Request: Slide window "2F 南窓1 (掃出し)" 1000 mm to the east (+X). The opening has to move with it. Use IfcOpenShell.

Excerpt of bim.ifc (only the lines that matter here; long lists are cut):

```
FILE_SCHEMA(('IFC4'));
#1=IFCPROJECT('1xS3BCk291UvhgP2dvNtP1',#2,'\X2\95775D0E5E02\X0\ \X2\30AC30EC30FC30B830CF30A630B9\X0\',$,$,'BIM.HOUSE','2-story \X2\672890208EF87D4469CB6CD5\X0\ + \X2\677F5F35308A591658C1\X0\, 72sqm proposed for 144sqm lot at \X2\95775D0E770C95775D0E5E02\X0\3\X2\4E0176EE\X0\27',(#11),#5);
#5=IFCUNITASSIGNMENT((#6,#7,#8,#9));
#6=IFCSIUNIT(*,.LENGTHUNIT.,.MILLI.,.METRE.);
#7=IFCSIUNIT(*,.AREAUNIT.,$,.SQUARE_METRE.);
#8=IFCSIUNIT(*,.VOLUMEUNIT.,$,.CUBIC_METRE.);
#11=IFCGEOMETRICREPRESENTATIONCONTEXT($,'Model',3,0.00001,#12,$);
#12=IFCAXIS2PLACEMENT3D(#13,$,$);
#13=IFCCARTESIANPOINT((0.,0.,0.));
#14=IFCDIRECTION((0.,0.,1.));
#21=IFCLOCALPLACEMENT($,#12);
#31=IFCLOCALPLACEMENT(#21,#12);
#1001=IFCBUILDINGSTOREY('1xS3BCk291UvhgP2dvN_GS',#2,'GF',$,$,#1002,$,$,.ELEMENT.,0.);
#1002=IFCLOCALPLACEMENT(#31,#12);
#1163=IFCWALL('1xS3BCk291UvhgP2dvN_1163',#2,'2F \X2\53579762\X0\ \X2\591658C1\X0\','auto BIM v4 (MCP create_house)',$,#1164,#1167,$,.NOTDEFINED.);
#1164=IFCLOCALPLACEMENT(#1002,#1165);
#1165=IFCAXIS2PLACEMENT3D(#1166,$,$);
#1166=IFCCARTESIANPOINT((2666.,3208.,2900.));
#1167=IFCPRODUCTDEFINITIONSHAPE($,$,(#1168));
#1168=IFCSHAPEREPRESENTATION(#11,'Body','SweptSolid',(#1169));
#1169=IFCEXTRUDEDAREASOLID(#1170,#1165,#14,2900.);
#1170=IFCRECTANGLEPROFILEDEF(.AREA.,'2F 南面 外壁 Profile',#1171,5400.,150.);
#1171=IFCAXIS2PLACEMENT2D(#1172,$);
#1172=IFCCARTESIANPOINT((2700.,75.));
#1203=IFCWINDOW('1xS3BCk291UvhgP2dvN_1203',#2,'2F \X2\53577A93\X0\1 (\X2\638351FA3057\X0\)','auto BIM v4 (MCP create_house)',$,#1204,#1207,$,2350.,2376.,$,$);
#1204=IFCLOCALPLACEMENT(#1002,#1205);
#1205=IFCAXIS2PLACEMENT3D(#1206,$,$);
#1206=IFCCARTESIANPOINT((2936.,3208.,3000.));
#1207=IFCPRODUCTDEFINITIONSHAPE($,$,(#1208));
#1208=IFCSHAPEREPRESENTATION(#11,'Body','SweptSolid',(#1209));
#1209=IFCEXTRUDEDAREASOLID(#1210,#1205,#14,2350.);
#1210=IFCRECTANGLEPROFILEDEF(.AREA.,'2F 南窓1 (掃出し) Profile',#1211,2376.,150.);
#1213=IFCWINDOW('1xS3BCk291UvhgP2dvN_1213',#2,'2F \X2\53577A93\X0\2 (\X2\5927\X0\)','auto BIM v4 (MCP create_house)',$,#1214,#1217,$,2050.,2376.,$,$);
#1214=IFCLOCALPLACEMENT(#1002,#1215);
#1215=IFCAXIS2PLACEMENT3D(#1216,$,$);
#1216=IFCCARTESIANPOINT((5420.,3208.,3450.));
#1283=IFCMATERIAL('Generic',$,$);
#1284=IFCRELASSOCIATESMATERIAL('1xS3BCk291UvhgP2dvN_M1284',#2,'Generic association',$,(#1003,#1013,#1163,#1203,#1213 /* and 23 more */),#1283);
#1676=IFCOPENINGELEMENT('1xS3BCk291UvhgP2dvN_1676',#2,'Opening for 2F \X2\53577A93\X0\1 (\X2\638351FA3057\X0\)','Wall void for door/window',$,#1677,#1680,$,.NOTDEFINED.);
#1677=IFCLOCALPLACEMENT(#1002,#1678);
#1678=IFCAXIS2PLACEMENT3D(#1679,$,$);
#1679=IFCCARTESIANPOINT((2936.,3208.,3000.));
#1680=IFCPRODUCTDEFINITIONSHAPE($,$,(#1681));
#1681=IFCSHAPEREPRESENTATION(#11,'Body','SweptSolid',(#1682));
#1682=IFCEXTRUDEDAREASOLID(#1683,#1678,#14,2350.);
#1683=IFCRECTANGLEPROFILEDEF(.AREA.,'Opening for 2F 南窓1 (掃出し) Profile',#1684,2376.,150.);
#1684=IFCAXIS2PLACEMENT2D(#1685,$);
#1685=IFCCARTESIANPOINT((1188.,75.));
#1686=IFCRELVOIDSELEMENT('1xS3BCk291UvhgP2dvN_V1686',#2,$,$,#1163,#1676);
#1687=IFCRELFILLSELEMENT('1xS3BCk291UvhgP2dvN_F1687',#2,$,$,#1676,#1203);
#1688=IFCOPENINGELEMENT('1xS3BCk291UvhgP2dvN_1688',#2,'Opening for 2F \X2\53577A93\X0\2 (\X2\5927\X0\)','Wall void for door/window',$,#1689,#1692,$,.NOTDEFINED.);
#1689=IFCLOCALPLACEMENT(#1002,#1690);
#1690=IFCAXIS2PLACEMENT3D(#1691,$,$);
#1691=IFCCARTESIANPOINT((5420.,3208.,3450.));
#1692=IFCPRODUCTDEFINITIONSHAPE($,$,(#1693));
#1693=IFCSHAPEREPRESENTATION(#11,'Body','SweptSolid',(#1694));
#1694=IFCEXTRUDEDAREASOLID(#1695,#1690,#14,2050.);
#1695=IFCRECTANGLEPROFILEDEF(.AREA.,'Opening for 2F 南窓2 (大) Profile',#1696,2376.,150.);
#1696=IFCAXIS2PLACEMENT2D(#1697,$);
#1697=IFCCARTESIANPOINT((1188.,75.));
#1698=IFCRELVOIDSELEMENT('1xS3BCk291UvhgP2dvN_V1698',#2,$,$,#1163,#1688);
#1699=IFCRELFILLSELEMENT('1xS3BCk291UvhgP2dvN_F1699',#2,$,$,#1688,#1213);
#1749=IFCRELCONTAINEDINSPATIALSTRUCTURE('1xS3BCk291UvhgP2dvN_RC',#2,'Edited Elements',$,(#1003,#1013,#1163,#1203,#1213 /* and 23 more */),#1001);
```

```python
import ifcopenshell
import ifcopenshell.api.geometry
import ifcopenshell.util.placement

model = ifcopenshell.open("bim.ifc")

window = model.by_guid("1xS3BCk291UvhgP2dvN_1203")
opening = window.FillsVoids[0].RelatingOpeningElement
wall = opening.VoidsElements[0].RelatingBuildingElement

wall_matrix = ifcopenshell.util.placement.get_local_placement(wall.ObjectPlacement)
shift = wall_matrix[:3, 0] * 1000.0
before = ifcopenshell.util.placement.get_local_placement(window.ObjectPlacement)[:3, 3].copy()

# The window is not placed relative to its opening, so move both.
for product in (opening, window):
    matrix = ifcopenshell.util.placement.get_local_placement(product.ObjectPlacement)
    matrix[:3, 3] += shift
    ifcopenshell.api.geometry.edit_object_placement(model, product=product, matrix=matrix, is_si=False)

after = ifcopenshell.util.placement.get_local_placement(window.ObjectPlacement)[:3, 3]
print("window moved by", (after - before).round(3) + 0.0)

model.write("bim_edited.ifc")
```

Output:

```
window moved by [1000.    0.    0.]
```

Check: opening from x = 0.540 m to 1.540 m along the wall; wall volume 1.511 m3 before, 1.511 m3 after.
